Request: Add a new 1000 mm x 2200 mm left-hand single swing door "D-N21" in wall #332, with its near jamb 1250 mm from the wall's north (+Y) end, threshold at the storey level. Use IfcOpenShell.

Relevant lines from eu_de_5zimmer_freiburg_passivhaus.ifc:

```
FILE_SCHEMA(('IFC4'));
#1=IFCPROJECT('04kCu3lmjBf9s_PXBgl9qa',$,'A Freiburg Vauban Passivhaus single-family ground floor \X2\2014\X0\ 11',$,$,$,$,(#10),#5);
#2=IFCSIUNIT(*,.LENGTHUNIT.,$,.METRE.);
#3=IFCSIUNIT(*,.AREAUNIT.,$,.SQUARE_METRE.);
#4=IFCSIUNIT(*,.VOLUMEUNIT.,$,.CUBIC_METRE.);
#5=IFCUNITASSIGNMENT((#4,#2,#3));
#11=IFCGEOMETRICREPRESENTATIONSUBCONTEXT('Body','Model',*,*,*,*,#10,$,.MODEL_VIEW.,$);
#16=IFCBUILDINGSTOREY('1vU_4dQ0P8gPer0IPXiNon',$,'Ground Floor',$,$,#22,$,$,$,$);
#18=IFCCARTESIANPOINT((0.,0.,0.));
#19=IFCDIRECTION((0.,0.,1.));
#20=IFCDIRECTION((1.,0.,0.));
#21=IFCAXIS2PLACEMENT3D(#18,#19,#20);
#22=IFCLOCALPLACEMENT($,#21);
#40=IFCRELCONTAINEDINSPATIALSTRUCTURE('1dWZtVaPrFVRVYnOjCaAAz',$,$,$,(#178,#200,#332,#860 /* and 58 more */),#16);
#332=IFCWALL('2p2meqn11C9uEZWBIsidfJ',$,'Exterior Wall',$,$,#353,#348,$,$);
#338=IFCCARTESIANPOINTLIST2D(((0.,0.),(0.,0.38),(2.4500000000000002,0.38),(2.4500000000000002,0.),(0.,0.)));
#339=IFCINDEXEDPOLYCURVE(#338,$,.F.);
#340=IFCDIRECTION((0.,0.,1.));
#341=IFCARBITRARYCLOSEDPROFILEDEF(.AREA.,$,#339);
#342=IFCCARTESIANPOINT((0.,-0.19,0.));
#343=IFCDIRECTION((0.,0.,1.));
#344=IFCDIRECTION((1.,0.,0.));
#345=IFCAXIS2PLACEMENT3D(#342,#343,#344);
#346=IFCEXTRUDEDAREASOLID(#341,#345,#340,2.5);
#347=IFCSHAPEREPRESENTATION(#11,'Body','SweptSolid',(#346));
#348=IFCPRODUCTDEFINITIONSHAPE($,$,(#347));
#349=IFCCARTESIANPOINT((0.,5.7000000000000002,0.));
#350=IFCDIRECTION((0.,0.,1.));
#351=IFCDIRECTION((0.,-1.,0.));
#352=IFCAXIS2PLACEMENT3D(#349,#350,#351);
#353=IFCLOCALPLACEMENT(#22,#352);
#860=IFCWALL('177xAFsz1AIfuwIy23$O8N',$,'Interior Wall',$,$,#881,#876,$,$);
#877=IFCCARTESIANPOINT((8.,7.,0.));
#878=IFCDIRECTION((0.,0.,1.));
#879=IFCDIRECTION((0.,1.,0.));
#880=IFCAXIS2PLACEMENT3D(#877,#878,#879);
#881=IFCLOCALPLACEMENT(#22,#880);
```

```python
import numpy as np
import ifcopenshell
import ifcopenshell.api.feature
import ifcopenshell.api.geometry
import ifcopenshell.api.root
import ifcopenshell.api.spatial
import ifcopenshell.geom
import ifcopenshell.util.element
import ifcopenshell.util.placement
import ifcopenshell.util.representation
import ifcopenshell.util.shape
import ifcopenshell.util.unit

model = ifcopenshell.open("eu_de_5zimmer_freiburg_passivhaus.ifc")
unit_scale = ifcopenshell.util.unit.calculate_unit_scale(model)
settings = ifcopenshell.geom.settings()


def volume(element):
    """Net volume in cubic metres, openings subtracted."""
    shape = ifcopenshell.geom.create_shape(settings, element)
    return ifcopenshell.util.shape.get_volume(shape.geometry)


wall = model.by_id(332)
storey = ifcopenshell.util.element.get_container(wall, ifc_class="IfcBuildingStorey")
context = ifcopenshell.util.representation.get_context(model, "Model", "Body", "MODEL_VIEW")
before = volume(wall)

width, height, from_end, sill = 1, 2.2, 1.25, 0.0  # metres

# The wall runs along its own X axis, and the end named is its -X end.
wall_shape = ifcopenshell.geom.create_shape(settings, wall)
x, y, z = ifcopenshell.util.shape.get_vertices(wall_shape.geometry).T
start = x.min() + from_end
face, thickness = float(y.min()), float(y.max() - y.min())
wall_matrix = ifcopenshell.util.placement.get_local_placement(wall.ObjectPlacement)
level = ifcopenshell.util.placement.get_local_placement(storey.ObjectPlacement)[2, 3]


def in_wall(x, y):
    """Placement at x, y metres in the wall's axes, at sill height."""
    matrix = wall_matrix.copy()
    matrix[:, 3] = wall_matrix @ np.array([x / unit_scale, y / unit_scale, 0.0, 1.0])
    matrix[2, 3] = level + sill / unit_scale
    return matrix


# Opening: a box that overshoots both wall faces by 50 mm.
opening = ifcopenshell.api.root.create_entity(model, ifc_class="IfcOpeningElement", predefined_type="OPENING")
box = ifcopenshell.api.geometry.add_wall_representation(
    model, context=context, length=width, height=height, thickness=thickness + 0.1
)
ifcopenshell.api.geometry.assign_representation(model, product=opening, representation=box)
ifcopenshell.api.geometry.edit_object_placement(model, product=opening, matrix=in_wall(start, face - 0.05), is_si=False)
ifcopenshell.api.feature.add_feature(model, feature=opening, element=wall)

door = ifcopenshell.api.root.create_entity(model, ifc_class="IfcDoor", name="D-N21", predefined_type="DOOR")
door.OverallWidth, door.OverallHeight = width / unit_scale, height / unit_scale
door.OperationType = "SINGLE_SWING_LEFT"
body = ifcopenshell.api.geometry.add_door_representation(
    model,
    context=context,
    overall_width=door.OverallWidth,
    overall_height=door.OverallHeight,
    operation_type="SINGLE_SWING_LEFT",
    lining_properties={"LiningDepth": thickness / unit_scale, "ThresholdDepth": thickness / unit_scale},
)
ifcopenshell.api.geometry.assign_representation(model, product=door, representation=body)
ifcopenshell.api.spatial.assign_container(model, products=[door], relating_structure=storey)
ifcopenshell.api.feature.add_filling(model, opening=opening, element=door)

# The lining spans the wall, so the door starts at the wall face.
ifcopenshell.api.geometry.edit_object_placement(model, product=door, matrix=in_wall(start, face), is_si=False)

after = volume(wall)

print(f"wall volume {before:.3f} -> {after:.3f} m3")

model.write("eu_de_5zimmer_freiburg_passivhaus-out.ifc")
```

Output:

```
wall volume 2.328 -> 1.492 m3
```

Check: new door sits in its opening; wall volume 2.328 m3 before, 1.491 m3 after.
